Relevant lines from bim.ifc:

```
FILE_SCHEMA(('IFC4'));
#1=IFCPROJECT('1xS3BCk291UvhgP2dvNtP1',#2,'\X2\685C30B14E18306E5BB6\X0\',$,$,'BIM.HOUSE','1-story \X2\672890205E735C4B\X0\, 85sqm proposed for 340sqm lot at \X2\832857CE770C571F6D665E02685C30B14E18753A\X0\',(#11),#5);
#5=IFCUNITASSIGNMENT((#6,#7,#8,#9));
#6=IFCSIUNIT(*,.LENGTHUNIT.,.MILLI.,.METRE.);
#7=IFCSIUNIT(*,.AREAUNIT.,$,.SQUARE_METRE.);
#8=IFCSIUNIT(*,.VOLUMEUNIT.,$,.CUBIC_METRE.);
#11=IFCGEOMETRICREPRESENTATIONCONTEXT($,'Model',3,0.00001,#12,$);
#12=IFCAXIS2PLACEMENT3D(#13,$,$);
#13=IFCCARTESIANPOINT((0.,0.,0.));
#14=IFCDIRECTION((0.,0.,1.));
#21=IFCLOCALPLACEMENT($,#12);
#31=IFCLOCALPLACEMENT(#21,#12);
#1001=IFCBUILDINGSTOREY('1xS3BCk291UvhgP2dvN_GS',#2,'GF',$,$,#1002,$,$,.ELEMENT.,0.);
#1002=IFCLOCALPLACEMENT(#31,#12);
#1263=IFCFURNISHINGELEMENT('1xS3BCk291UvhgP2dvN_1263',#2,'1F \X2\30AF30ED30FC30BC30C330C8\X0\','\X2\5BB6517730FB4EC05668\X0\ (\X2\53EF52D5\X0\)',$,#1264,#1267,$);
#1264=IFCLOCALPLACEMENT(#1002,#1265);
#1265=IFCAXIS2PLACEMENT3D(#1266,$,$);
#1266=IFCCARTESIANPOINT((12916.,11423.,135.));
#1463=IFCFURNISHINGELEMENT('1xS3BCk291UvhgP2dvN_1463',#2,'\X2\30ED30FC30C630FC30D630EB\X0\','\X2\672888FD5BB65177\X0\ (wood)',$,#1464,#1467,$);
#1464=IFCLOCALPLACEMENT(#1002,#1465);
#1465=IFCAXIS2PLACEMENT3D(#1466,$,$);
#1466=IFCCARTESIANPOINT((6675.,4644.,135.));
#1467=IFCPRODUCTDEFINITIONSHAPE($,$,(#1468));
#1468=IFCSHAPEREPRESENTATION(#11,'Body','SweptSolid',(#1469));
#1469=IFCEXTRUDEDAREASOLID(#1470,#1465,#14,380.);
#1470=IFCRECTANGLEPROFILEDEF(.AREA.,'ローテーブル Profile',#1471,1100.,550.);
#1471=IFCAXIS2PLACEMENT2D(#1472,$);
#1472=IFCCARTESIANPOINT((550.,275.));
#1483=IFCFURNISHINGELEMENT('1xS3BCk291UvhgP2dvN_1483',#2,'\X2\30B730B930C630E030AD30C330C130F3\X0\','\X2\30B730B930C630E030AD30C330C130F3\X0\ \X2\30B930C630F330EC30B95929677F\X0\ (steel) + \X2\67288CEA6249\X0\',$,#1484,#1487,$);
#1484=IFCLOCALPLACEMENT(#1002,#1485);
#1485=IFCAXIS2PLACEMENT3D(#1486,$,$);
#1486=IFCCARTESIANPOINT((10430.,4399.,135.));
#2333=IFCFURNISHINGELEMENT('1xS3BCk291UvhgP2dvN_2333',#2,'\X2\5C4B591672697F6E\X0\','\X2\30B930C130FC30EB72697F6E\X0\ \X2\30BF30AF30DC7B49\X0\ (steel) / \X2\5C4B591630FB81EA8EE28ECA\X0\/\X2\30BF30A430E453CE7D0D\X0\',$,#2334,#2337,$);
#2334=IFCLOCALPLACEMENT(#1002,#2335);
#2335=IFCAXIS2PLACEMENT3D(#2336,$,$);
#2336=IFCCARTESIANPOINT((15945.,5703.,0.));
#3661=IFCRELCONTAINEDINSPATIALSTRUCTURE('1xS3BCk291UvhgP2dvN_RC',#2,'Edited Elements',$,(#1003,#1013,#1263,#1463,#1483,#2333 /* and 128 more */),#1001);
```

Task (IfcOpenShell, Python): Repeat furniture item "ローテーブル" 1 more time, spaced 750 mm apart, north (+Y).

```python
import numpy as np
import ifcopenshell
import ifcopenshell.api.geometry
import ifcopenshell.api.root
import ifcopenshell.util.element
import ifcopenshell.util.placement
import ifcopenshell.util.unit

model = ifcopenshell.open("bim.ifc")
unit_scale = ifcopenshell.util.unit.calculate_unit_scale(model)


def reuse_history(source, copy):
    """copy_class also copies each property set's owner history, people and application; keep the originals."""
    for rel in copy.IsDefinedBy:
        if rel.is_a("IfcRelDefinesByProperties") and (history := rel.RelatingPropertyDefinition.OwnerHistory):
            rel.RelatingPropertyDefinition.OwnerHistory = source.OwnerHistory
            ifcopenshell.util.element.remove_deep2(model, history)


source = model.by_id(1463)
base = ifcopenshell.util.placement.get_local_placement(source.ObjectPlacement)
step = np.array([0.0, 1.0, 0.0]) * 0.75 / unit_scale

for i in range(1, 2):
    copy = ifcopenshell.api.root.copy_class(model, product=source)
    copy.Representation = ifcopenshell.util.element.copy_deep(
        model, source.Representation, exclude=["IfcGeometricRepresentationContext", "IfcRepresentationMap"]
    )
    reuse_history(source, copy)
    matrix = base.copy()
    matrix[:3, 3] += i * step
    print("added at", matrix[:3, 3].round(3) + 0.0)
    ifcopenshell.api.geometry.edit_object_placement(model, product=copy, matrix=matrix, is_si=False)

model.write("bim-out.ifc")
```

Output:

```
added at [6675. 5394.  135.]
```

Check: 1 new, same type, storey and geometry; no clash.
